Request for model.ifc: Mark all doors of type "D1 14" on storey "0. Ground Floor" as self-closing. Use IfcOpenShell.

First a look at what the model holds.

```python
import ifcopenshell
import ifcopenshell.util.element

model = ifcopenshell.open("model.ifc")
print(model.schema)
storey = next(s for s in model.by_type("IfcBuildingStorey") if s.Name == "0. Ground Floor")
doors = [e for e in ifcopenshell.util.element.get_decomposition(storey) if e.is_a("IfcDoor")]
seen = {}
for e in doors:
    element_type = ifcopenshell.util.element.get_type(e)
    key = (element_type.Name if element_type != e and element_type else None, ifcopenshell.util.element.get_pset(e, "Pset_DoorCommon", "SelfClosing"))
    seen[key] = seen.get(key, 0) + 1
for (name, value), count in sorted(seen.items(), key=str):
    print(count, "x", name, "|", value)
```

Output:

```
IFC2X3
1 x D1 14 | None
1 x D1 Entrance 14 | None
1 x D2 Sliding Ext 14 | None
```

```python
import ifcopenshell
import ifcopenshell.api.pset
import ifcopenshell.util.element

model = ifcopenshell.open("model.ifc")

storey = next(s for s in model.by_type("IfcBuildingStorey") if s.Name == "0. Ground Floor")
doors = [e for e in ifcopenshell.util.element.get_decomposition(storey) if e.is_a("IfcDoor")]

count = 0
for e in doors:
    element_type = ifcopenshell.util.element.get_type(e)
    if element_type in (None, e) or element_type.Name != "D1 14":
        continue
    # add_pset returns the element's existing set when there is one.
    pset = ifcopenshell.api.pset.add_pset(model, product=e, name="Pset_DoorCommon")
    ifcopenshell.api.pset.edit_pset(model, pset=pset, properties={"SelfClosing": True})
    count += 1

print(count, "doors updated")

model.write("model-out.ifc")
```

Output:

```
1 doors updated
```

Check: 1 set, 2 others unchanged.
